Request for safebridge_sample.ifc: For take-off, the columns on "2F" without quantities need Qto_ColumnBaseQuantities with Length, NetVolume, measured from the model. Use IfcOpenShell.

First a look at what the model holds.

```python
import ifcopenshell
import ifcopenshell.util.element
import ifcopenshell.util.unit

model = ifcopenshell.open("safebridge_sample.ifc")
print(model.schema)
for unit_type in ("LENGTHUNIT", "AREAUNIT", "VOLUMEUNIT"):
    print(unit_type, ifcopenshell.util.unit.calculate_unit_scale(model, unit_type))
storey = next(s for s in model.by_type("IfcBuildingStorey") if s.Name == "2F")
columns = [e for e in ifcopenshell.util.element.get_decomposition(storey) if e.is_a("IfcColumn")]
for e in sorted(columns, key=lambda e: e.id()):
    print(e.id(), e.is_a(), e.Name, list(ifcopenshell.util.element.get_psets(e, qtos_only=True)), sep=" | ")
```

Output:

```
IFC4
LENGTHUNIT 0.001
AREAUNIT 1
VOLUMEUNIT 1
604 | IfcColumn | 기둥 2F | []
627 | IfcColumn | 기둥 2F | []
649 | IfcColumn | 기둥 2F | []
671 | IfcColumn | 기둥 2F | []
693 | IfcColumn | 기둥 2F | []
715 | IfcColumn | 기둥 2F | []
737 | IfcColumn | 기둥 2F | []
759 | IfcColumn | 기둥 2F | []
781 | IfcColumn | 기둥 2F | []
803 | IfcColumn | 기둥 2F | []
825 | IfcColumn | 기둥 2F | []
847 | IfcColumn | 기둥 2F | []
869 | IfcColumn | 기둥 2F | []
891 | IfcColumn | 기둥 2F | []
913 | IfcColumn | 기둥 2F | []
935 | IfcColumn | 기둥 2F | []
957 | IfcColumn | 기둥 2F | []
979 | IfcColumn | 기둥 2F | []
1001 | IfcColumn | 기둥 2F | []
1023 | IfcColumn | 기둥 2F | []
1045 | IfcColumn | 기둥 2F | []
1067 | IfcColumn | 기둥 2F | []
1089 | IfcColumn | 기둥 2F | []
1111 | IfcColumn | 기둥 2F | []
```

```python
import ifcopenshell
import ifcopenshell.api.pset
import ifcopenshell.geom
import ifcopenshell.util.element
import ifcopenshell.util.shape
import ifcopenshell.util.unit

model = ifcopenshell.open("safebridge_sample.ifc")
unit_scale = ifcopenshell.util.unit.calculate_unit_scale(model)
volume_scale = ifcopenshell.util.unit.calculate_unit_scale(model, "VOLUMEUNIT")
settings = ifcopenshell.geom.settings()

storey = next(s for s in model.by_type("IfcBuildingStorey") if s.Name == "2F")
columns = [e for e in ifcopenshell.util.element.get_decomposition(storey) if e.is_a("IfcColumn")]

for e in sorted(columns, key=lambda e: e.id()):
    if ifcopenshell.util.element.get_psets(e, qtos_only=True, should_inherit=False):
        continue
    # Geometry comes back in metres, in the element's own axes.
    shape = ifcopenshell.geom.create_shape(settings, e)
    values = {
        "Length": ifcopenshell.util.shape.get_z(shape.geometry) / unit_scale,
        "NetVolume": ifcopenshell.util.shape.get_volume(shape.geometry) / volume_scale,
    }
    qto = ifcopenshell.api.pset.add_qto(model, product=e, name="Qto_ColumnBaseQuantities")
    ifcopenshell.api.pset.edit_qto(model, qto=qto, properties=values)
    print(e.id(), {k: round(v, 3) for k, v in values.items()})

model.write("safebridge_sample_rev.ifc")
```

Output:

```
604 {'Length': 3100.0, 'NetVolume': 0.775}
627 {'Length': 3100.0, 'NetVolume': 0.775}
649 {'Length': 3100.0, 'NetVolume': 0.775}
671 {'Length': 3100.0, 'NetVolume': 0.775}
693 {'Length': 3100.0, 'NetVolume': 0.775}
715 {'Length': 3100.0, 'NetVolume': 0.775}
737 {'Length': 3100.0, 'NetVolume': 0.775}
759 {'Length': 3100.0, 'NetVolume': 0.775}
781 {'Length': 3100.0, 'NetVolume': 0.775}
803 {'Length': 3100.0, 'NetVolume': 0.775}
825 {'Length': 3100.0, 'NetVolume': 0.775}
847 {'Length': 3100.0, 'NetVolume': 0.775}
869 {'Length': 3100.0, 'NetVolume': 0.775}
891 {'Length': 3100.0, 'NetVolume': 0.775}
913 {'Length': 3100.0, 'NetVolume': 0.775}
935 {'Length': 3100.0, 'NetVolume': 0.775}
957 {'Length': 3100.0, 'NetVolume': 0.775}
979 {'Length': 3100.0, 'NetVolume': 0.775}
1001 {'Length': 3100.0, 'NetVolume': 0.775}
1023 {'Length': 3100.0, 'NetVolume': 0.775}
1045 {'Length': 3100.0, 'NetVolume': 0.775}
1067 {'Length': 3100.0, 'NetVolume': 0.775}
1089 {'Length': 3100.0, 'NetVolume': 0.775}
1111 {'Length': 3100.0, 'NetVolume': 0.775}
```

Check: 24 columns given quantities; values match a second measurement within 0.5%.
